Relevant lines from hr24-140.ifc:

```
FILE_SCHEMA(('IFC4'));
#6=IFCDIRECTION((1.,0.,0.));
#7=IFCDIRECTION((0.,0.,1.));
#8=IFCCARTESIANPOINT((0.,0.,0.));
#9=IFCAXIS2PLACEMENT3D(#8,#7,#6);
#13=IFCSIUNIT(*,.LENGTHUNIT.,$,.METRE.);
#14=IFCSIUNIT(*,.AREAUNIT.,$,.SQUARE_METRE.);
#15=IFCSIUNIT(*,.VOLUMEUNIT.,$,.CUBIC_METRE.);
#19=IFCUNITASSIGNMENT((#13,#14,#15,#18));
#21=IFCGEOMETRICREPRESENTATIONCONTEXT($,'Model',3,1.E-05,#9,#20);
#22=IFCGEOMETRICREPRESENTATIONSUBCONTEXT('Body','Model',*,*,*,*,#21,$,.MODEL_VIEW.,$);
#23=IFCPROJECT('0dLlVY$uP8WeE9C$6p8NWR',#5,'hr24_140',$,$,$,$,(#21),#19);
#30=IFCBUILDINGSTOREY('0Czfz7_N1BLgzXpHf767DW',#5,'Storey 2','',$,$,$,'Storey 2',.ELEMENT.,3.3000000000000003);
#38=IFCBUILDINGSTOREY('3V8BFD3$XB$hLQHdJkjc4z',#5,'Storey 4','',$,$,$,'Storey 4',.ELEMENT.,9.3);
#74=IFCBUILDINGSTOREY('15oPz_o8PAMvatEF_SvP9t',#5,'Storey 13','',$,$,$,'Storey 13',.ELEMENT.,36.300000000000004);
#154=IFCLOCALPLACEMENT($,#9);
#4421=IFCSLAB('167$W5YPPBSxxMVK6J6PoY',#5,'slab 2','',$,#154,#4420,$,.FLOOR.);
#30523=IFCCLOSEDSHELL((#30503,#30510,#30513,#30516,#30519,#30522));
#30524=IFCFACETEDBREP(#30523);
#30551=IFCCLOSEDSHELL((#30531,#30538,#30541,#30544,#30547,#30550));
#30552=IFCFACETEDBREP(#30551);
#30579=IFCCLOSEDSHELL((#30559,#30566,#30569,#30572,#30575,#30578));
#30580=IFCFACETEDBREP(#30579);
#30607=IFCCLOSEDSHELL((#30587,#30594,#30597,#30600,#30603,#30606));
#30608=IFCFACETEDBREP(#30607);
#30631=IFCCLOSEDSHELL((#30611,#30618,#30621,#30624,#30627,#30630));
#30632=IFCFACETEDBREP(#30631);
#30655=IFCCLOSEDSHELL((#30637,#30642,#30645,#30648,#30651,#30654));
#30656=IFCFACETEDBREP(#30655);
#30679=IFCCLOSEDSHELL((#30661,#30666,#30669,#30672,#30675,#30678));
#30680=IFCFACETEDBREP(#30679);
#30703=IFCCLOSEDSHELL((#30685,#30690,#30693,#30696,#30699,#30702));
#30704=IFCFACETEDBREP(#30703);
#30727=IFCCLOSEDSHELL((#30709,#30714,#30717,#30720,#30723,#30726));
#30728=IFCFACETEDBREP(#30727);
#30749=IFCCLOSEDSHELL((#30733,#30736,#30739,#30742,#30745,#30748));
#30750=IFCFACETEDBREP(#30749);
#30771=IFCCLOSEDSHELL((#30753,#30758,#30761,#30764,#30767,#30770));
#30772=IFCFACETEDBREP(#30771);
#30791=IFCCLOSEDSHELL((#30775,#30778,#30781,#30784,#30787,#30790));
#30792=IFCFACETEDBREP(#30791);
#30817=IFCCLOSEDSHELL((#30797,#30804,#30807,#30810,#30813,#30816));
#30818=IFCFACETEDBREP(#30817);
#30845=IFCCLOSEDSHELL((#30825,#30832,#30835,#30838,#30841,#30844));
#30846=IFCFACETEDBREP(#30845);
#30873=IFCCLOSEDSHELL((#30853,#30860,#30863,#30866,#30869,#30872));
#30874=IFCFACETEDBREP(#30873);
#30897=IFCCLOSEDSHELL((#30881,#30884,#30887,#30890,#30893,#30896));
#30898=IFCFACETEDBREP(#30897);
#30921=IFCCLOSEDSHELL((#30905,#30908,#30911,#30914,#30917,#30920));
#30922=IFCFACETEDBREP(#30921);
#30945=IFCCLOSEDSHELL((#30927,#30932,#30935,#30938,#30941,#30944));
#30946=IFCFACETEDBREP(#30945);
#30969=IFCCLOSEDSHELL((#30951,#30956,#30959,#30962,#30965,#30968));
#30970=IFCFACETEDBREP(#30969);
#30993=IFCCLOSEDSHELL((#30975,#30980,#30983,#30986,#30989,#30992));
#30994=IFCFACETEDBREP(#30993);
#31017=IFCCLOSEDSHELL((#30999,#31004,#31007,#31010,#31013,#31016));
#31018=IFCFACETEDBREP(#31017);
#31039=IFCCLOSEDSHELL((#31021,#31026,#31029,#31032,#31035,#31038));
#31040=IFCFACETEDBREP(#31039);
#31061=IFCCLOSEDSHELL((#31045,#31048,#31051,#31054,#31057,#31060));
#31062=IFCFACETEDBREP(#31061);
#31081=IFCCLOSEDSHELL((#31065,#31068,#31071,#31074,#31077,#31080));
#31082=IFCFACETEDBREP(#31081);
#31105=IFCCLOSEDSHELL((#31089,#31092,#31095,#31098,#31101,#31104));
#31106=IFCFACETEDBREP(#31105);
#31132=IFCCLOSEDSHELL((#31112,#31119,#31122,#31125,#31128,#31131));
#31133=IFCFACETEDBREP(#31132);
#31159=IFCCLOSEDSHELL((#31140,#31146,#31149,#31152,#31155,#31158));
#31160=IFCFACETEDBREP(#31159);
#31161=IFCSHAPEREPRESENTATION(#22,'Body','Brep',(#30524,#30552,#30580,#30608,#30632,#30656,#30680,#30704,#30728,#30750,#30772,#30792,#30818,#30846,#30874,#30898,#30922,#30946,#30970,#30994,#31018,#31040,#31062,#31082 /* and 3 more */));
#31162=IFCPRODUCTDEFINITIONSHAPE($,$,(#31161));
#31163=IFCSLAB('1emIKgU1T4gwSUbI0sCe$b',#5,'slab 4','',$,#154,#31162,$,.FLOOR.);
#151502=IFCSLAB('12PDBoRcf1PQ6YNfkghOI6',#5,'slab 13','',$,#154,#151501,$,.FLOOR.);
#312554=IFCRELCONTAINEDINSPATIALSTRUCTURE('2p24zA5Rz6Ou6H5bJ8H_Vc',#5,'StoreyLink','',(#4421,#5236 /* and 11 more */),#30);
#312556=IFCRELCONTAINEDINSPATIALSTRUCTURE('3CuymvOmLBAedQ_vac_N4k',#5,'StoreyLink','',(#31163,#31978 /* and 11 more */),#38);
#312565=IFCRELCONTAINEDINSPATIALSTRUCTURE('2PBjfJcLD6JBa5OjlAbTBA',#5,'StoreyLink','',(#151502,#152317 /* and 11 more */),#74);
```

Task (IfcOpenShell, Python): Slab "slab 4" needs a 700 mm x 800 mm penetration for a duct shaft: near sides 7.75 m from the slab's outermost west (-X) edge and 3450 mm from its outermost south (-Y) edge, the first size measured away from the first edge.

```python
import numpy as np
import ifcopenshell
import ifcopenshell.api.feature
import ifcopenshell.api.geometry
import ifcopenshell.api.root
import ifcopenshell.geom
import ifcopenshell.util.placement
import ifcopenshell.util.representation
import ifcopenshell.util.shape
import ifcopenshell.util.unit

model = ifcopenshell.open("hr24-140.ifc")
unit_scale = ifcopenshell.util.unit.calculate_unit_scale(model)
settings = ifcopenshell.geom.settings()


def volume(element):
    """Net volume in cubic metres, openings subtracted."""
    shape = ifcopenshell.geom.create_shape(settings, element)
    return ifcopenshell.util.shape.get_volume(shape.geometry)


slab = model.by_guid("1emIKgU1T4gwSUbI0sCe$b")
before = volume(slab)

# Extent in the slab's own axes, in metres. The edges named are its -X and -Y sides.
slab_shape = ifcopenshell.geom.create_shape(settings, slab)
vertices = ifcopenshell.util.shape.get_vertices(slab_shape.geometry)
x_min, y_min, bottom = vertices.min(axis=0)
top = vertices[:, 2].max()

opening = ifcopenshell.api.root.create_entity(model, ifc_class="IfcOpeningElement", name="Duct shaft opening", predefined_type="OPENING")
context = ifcopenshell.util.representation.get_context(model, "Model", "Body", "MODEL_VIEW")
width, depth = 0.7, 0.8
outline = [(0.0, 0.0), (width, 0.0), (width, depth), (0.0, depth), (0.0, 0.0)]
# Overshoot both faces by 50 mm so the cut is clean.
shape = ifcopenshell.api.geometry.add_slab_representation(
    model, context=context, depth=top - bottom + 0.1, polyline=outline
)
ifcopenshell.api.geometry.assign_representation(model, product=opening, representation=shape)

matrix = ifcopenshell.util.placement.get_local_placement(slab.ObjectPlacement)
matrix[:, 3] = matrix @ np.append(np.array([x_min + 7.75, y_min + 3.45, bottom - 0.05]) / unit_scale, 1.0)
ifcopenshell.api.geometry.edit_object_placement(model, product=opening, matrix=matrix, is_si=False)
ifcopenshell.api.feature.add_feature(model, feature=opening, element=slab)

after = volume(slab)

print(f"slab volume {before:.3f} -> {after:.3f} m3")

model.write("hr24-140_rev.ifc")
```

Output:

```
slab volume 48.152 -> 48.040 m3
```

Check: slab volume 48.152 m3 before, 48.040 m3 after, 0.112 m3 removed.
